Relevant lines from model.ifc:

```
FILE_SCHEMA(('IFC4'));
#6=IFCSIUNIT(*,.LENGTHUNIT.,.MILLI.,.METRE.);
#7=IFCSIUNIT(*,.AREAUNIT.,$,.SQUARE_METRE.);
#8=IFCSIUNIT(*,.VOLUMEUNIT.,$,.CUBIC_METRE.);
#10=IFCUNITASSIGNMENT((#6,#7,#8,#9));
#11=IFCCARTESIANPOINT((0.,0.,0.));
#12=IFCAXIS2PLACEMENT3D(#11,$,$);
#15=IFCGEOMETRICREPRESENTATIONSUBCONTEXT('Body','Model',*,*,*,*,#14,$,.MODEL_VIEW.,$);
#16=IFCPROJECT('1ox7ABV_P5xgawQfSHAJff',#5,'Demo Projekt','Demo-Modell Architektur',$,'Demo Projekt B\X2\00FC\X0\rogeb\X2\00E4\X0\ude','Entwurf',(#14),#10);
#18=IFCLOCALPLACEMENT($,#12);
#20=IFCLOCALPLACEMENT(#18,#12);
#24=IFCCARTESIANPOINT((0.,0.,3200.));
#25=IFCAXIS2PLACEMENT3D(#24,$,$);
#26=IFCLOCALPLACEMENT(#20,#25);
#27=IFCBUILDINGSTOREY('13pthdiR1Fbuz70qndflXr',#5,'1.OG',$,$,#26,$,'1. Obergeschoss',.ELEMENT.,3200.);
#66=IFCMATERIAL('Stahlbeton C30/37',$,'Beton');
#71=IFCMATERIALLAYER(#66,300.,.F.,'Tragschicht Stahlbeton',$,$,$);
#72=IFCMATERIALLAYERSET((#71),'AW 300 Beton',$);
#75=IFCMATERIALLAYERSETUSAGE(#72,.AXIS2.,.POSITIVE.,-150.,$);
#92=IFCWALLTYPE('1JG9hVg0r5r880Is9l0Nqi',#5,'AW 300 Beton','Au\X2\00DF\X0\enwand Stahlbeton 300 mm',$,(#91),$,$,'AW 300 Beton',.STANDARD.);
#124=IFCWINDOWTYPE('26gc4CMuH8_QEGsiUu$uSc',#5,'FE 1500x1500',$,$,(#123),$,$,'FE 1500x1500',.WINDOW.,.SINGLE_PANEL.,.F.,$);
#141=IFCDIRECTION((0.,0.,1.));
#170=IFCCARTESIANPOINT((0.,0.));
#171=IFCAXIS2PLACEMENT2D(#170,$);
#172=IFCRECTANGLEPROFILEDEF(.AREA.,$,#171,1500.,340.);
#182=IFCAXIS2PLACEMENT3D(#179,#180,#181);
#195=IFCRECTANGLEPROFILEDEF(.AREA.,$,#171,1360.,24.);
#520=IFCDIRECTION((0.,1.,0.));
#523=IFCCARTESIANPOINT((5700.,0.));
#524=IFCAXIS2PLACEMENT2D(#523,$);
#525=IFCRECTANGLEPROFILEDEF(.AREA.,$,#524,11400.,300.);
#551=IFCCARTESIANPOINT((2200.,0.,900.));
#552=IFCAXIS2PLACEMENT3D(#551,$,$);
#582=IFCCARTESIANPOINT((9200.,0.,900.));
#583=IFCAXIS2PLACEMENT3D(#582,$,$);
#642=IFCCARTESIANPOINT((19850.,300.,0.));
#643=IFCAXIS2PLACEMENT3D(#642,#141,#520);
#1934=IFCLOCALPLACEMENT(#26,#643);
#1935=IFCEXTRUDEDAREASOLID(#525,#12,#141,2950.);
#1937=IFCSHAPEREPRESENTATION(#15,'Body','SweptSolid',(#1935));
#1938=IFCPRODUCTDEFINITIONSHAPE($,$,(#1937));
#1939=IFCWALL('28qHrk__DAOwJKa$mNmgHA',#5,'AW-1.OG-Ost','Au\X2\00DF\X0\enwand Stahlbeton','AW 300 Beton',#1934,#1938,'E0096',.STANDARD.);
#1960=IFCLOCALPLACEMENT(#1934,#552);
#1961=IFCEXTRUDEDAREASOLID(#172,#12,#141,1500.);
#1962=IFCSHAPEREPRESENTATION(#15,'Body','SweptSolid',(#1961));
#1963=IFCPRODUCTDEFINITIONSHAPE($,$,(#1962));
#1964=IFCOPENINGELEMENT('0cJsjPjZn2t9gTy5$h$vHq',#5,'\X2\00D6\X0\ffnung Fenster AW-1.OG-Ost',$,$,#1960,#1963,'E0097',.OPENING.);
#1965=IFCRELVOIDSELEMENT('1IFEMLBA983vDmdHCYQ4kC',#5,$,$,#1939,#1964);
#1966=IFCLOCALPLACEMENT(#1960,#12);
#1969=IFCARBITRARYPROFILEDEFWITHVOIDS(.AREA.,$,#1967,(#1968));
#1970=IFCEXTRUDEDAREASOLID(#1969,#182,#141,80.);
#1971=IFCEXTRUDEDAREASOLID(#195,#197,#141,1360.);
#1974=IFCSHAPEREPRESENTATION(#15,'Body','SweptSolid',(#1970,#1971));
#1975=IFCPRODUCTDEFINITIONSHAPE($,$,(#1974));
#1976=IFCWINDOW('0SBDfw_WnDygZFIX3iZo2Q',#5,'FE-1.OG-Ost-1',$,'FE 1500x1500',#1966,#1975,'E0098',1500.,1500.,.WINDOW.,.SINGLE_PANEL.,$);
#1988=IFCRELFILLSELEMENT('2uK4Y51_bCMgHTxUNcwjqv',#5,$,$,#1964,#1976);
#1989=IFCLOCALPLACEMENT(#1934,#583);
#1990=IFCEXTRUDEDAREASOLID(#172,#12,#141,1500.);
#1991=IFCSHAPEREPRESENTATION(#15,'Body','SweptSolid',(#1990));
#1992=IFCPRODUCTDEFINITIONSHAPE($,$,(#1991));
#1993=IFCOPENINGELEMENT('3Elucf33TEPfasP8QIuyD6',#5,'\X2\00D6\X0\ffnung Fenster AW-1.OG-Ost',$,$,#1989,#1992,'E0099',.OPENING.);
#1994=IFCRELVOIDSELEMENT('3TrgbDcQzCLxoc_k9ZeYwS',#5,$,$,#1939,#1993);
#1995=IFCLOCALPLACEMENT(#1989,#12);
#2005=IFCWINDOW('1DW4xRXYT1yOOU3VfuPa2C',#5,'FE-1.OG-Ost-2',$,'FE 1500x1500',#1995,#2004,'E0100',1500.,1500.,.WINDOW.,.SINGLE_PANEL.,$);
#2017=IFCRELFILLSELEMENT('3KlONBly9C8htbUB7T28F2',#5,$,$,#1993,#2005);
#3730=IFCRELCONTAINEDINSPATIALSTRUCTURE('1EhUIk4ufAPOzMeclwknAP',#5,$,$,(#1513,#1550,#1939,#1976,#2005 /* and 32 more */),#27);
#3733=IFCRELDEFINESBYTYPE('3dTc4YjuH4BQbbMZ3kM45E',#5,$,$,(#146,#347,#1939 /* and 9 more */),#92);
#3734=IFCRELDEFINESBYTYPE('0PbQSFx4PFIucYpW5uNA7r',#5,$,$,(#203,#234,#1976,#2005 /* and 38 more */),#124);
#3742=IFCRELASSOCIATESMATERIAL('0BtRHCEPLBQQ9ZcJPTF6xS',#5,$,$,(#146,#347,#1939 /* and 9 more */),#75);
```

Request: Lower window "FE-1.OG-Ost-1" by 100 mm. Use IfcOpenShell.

```python
import numpy as np
import ifcopenshell
import ifcopenshell.api.geometry
import ifcopenshell.util.placement
import ifcopenshell.util.unit

model = ifcopenshell.open("model.ifc")
unit_scale = ifcopenshell.util.unit.calculate_unit_scale(model)

window = model.by_guid("0SBDfw_WnDygZFIX3iZo2Q")
opening = window.FillsVoids[0].RelatingOpeningElement
dz = -0.1 / unit_scale

shift = np.array([0.0, 0.0, dz])
# The window is placed relative to its opening, so it follows when the opening moves.
matrix = ifcopenshell.util.placement.get_local_placement(opening.ObjectPlacement)
matrix[:3, 3] += shift
ifcopenshell.api.geometry.edit_object_placement(
    model, product=opening, matrix=matrix, is_si=False, should_transform_children=True
)

print(f"moved by {dz * unit_scale:+.3f} m")

model.write("model-out.ifc")
```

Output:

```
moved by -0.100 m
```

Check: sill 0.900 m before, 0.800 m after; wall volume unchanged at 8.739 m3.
